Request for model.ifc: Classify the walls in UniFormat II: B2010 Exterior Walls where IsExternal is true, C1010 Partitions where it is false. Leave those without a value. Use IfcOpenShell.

First a look at what the model holds.

```python
import ifcopenshell
import ifcopenshell.util.element

model = ifcopenshell.open("model.ifc")
print(model.schema)
print("classifications:", [c.Name for c in model.by_type("IfcClassification")])
values = [ifcopenshell.util.element.get_pset(e, "Pset_WallCommon", "IsExternal") for e in model.by_type("IfcWall")]
for value in (True, False, None):
    print("IsExternal", value, values.count(value))
```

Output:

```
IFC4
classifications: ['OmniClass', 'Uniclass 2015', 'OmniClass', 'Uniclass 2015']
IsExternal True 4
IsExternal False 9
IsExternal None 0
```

```python
import ifcopenshell
import ifcopenshell.api.classification
import ifcopenshell.util.element

model = ifcopenshell.open("model.ifc")

system = ifcopenshell.api.classification.add_classification(model, classification="UniFormat II")

walls = model.by_type("IfcWall")
external = {e: ifcopenshell.util.element.get_pset(e, "Pset_WallCommon", "IsExternal") for e in walls}
for flag, code, name in ((True, "B2010", "Exterior Walls"), (False, "C1010", "Partitions")):
    products = [e for e in walls if external[e] is flag]
    ifcopenshell.api.classification.add_reference(
        model, products=products, classification=system, identification=code, name=name
    )
    print(code, len(products))

model.write("model-out.ifc")
```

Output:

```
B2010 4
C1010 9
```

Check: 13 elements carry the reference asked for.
